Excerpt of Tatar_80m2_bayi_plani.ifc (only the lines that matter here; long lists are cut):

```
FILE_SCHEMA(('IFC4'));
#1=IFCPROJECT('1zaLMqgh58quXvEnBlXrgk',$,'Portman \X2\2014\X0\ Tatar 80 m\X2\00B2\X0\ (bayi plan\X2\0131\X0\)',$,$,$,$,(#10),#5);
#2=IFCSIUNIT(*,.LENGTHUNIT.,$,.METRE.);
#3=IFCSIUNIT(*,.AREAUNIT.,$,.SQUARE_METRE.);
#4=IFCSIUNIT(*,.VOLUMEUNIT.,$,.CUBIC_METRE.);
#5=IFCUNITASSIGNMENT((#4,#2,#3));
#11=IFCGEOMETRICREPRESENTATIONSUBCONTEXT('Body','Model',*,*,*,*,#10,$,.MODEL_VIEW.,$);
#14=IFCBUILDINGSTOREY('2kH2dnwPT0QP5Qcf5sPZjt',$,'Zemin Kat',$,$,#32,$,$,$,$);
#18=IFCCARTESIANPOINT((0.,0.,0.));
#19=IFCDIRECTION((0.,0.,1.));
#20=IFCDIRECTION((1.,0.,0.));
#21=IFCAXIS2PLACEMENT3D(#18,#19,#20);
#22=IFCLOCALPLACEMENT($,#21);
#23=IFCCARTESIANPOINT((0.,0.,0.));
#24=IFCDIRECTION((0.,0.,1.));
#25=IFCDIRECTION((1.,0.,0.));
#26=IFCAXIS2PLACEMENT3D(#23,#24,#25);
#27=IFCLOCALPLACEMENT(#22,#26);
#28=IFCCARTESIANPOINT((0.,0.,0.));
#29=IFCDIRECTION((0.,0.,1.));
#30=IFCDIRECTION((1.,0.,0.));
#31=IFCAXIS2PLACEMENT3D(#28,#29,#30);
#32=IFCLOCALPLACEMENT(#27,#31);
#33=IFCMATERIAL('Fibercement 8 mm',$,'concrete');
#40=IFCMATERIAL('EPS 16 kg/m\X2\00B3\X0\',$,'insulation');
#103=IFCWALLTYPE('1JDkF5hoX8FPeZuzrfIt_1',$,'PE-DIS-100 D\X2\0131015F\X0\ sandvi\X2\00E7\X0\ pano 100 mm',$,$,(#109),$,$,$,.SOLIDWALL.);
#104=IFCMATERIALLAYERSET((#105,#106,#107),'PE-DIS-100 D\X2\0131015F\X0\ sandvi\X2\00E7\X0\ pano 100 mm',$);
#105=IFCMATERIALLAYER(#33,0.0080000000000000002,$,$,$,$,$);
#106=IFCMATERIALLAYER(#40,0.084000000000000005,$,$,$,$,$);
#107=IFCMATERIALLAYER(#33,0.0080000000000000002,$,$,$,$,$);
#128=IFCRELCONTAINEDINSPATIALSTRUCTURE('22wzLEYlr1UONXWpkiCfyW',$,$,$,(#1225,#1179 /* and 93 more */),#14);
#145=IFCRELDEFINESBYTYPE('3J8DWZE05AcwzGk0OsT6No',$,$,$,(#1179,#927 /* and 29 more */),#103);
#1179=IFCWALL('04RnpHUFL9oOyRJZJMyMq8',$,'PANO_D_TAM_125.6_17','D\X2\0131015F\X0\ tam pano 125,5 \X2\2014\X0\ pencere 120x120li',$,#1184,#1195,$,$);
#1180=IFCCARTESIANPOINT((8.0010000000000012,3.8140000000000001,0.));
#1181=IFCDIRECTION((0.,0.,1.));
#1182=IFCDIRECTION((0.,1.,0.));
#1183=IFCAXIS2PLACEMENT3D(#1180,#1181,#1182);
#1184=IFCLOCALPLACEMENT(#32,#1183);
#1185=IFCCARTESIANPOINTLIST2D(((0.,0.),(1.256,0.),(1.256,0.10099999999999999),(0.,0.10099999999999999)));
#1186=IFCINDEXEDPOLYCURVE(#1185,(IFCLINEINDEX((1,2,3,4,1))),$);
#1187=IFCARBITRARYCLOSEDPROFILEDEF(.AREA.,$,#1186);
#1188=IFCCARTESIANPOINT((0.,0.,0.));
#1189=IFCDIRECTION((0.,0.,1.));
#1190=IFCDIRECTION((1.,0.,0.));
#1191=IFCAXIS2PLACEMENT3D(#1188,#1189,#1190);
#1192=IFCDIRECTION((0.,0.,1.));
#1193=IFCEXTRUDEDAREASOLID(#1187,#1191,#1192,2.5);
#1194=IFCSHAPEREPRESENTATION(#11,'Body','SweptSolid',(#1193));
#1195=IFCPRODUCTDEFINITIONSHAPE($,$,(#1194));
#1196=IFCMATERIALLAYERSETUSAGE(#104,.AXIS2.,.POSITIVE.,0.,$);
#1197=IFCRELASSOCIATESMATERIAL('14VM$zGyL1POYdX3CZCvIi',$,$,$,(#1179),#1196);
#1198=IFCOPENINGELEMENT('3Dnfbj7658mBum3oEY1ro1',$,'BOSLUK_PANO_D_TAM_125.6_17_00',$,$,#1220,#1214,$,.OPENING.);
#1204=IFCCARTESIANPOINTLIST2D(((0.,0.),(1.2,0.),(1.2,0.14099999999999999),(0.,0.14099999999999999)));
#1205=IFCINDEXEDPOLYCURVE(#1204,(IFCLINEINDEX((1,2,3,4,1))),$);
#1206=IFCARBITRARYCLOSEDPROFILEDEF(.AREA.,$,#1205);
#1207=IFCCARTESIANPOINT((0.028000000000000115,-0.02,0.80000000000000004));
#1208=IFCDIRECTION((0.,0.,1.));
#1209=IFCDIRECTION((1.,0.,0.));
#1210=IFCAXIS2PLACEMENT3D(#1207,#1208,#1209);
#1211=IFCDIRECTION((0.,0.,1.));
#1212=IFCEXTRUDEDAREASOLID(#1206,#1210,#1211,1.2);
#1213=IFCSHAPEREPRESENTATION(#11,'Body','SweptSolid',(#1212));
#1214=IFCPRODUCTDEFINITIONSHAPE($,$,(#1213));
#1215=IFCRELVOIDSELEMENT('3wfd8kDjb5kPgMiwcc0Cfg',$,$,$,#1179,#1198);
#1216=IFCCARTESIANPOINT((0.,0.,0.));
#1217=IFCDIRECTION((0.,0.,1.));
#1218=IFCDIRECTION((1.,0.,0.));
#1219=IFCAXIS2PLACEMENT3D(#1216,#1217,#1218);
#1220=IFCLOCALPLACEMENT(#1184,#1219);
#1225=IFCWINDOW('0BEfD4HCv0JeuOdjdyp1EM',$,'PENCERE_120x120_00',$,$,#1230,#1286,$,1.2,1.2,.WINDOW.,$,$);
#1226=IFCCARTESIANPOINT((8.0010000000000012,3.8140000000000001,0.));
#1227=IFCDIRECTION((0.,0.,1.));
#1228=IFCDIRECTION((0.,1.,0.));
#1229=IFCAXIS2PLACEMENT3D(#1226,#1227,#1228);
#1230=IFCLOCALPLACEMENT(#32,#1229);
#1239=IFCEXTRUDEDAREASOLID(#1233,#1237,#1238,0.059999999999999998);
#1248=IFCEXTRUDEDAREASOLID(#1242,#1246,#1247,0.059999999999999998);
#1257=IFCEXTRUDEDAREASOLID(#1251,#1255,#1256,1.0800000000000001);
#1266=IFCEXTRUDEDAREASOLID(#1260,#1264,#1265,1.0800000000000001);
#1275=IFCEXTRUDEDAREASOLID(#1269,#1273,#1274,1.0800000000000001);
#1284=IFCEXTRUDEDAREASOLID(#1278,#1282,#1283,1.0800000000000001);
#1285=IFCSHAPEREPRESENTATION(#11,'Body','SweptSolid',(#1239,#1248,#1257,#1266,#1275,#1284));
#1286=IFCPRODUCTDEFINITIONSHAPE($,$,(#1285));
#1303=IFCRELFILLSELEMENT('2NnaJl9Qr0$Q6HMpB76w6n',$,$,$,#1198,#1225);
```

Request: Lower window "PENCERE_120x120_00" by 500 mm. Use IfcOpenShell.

```python
import numpy as np
import ifcopenshell
import ifcopenshell.api.geometry
import ifcopenshell.util.placement
import ifcopenshell.util.unit

model = ifcopenshell.open("Tatar_80m2_bayi_plani.ifc")
unit_scale = ifcopenshell.util.unit.calculate_unit_scale(model)

window = model.by_guid("0BEfD4HCv0JeuOdjdyp1EM")
opening = window.FillsVoids[0].RelatingOpeningElement
dz = -0.5 / unit_scale

shift = np.array([0.0, 0.0, dz])
# The window is not placed relative to its opening, so move both.
for product in (opening, window):
    matrix = ifcopenshell.util.placement.get_local_placement(product.ObjectPlacement)
    matrix[:3, 3] += shift
    ifcopenshell.api.geometry.edit_object_placement(model, product=product, matrix=matrix, is_si=False)

print(f"moved by {dz * unit_scale:+.3f} m")

model.write("Tatar_80m2_bayi_plani_rev.ifc")
```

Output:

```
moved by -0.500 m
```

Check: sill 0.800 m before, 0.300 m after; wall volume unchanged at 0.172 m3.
